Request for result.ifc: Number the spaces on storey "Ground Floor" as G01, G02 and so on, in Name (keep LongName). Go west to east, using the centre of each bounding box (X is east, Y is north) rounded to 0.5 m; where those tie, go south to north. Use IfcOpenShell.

First a look at what the model holds.

```python
import ifcopenshell
import ifcopenshell.util.element
import ifcopenshell.util.placement

model = ifcopenshell.open("result.ifc")
print(model.schema)
storey = next(s for s in model.by_type("IfcBuildingStorey") if s.Name == "Ground Floor")
spaces = [e for e in ifcopenshell.util.element.get_decomposition(storey) if e.is_a("IfcSpace")]
for e in sorted(spaces, key=lambda e: e.id()):
    origin = ifcopenshell.util.placement.get_local_placement(e.ObjectPlacement)[:3, 3]
    print(e.id(), e.Name, e.LongName, origin.round(2) + 0.0, sep=" | ")
```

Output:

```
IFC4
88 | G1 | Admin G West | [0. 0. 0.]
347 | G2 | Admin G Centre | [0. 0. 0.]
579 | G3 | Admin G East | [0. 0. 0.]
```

```python
import ifcopenshell
import ifcopenshell.geom
import ifcopenshell.util.element
import ifcopenshell.util.shape

model = ifcopenshell.open("result.ifc")
settings = ifcopenshell.geom.settings()
settings.set("use-world-coords", True)


def centre(element):
    shape = ifcopenshell.geom.create_shape(settings, element)
    return ifcopenshell.util.shape.get_bbox_centroid(shape.geometry)


storey = next(s for s in model.by_type("IfcBuildingStorey") if s.Name == "Ground Floor")
spaces = [e for e in ifcopenshell.util.element.get_decomposition(storey) if e.is_a("IfcSpace")]

# Insertion points can sit at a corner or the storey origin, so sort by the geometry (in metres).
centres = {e: centre(e) for e in spaces}
spaces.sort(key=lambda e: (round(centres[e][0] / 0.5), centres[e][1]))

for i, e in enumerate(spaces, start=1):
    number = f"G{i:02d}"
    e.Name = number
    print(e.id(), number)

model.write("result_v2.ifc")
```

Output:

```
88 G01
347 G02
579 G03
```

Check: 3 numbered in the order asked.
